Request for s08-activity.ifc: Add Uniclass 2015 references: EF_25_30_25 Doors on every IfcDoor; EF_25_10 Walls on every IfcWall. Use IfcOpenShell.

First a look at what the model holds.

```python
import ifcopenshell

model = ifcopenshell.open("s08-activity.ifc")
print(model.schema)
print("classifications:", [c.Name for c in model.by_type("IfcClassification")])
for ifc_class in ("IfcDoor", "IfcRoof", "IfcStair", "IfcWall", "IfcWindow"):
    print(ifc_class, len(model.by_type(ifc_class)))
```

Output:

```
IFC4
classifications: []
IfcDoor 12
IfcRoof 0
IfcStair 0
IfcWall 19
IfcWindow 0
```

```python
import ifcopenshell
import ifcopenshell.api.classification

model = ifcopenshell.open("s08-activity.ifc")

system = ifcopenshell.api.classification.add_classification(model, classification="Uniclass 2015")

codes = {
    "IfcDoor": ("EF_25_30_25", "Doors"),
    "IfcWall": ("EF_25_10", "Walls"),
}
for ifc_class, (code, name) in codes.items():
    products = model.by_type(ifc_class)
    ifcopenshell.api.classification.add_reference(
        model, products=products, classification=system, identification=code, name=name
    )
    print(code, len(products))

model.write("s08-activity_updated.ifc")
```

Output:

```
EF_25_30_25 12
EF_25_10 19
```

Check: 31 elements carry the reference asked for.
